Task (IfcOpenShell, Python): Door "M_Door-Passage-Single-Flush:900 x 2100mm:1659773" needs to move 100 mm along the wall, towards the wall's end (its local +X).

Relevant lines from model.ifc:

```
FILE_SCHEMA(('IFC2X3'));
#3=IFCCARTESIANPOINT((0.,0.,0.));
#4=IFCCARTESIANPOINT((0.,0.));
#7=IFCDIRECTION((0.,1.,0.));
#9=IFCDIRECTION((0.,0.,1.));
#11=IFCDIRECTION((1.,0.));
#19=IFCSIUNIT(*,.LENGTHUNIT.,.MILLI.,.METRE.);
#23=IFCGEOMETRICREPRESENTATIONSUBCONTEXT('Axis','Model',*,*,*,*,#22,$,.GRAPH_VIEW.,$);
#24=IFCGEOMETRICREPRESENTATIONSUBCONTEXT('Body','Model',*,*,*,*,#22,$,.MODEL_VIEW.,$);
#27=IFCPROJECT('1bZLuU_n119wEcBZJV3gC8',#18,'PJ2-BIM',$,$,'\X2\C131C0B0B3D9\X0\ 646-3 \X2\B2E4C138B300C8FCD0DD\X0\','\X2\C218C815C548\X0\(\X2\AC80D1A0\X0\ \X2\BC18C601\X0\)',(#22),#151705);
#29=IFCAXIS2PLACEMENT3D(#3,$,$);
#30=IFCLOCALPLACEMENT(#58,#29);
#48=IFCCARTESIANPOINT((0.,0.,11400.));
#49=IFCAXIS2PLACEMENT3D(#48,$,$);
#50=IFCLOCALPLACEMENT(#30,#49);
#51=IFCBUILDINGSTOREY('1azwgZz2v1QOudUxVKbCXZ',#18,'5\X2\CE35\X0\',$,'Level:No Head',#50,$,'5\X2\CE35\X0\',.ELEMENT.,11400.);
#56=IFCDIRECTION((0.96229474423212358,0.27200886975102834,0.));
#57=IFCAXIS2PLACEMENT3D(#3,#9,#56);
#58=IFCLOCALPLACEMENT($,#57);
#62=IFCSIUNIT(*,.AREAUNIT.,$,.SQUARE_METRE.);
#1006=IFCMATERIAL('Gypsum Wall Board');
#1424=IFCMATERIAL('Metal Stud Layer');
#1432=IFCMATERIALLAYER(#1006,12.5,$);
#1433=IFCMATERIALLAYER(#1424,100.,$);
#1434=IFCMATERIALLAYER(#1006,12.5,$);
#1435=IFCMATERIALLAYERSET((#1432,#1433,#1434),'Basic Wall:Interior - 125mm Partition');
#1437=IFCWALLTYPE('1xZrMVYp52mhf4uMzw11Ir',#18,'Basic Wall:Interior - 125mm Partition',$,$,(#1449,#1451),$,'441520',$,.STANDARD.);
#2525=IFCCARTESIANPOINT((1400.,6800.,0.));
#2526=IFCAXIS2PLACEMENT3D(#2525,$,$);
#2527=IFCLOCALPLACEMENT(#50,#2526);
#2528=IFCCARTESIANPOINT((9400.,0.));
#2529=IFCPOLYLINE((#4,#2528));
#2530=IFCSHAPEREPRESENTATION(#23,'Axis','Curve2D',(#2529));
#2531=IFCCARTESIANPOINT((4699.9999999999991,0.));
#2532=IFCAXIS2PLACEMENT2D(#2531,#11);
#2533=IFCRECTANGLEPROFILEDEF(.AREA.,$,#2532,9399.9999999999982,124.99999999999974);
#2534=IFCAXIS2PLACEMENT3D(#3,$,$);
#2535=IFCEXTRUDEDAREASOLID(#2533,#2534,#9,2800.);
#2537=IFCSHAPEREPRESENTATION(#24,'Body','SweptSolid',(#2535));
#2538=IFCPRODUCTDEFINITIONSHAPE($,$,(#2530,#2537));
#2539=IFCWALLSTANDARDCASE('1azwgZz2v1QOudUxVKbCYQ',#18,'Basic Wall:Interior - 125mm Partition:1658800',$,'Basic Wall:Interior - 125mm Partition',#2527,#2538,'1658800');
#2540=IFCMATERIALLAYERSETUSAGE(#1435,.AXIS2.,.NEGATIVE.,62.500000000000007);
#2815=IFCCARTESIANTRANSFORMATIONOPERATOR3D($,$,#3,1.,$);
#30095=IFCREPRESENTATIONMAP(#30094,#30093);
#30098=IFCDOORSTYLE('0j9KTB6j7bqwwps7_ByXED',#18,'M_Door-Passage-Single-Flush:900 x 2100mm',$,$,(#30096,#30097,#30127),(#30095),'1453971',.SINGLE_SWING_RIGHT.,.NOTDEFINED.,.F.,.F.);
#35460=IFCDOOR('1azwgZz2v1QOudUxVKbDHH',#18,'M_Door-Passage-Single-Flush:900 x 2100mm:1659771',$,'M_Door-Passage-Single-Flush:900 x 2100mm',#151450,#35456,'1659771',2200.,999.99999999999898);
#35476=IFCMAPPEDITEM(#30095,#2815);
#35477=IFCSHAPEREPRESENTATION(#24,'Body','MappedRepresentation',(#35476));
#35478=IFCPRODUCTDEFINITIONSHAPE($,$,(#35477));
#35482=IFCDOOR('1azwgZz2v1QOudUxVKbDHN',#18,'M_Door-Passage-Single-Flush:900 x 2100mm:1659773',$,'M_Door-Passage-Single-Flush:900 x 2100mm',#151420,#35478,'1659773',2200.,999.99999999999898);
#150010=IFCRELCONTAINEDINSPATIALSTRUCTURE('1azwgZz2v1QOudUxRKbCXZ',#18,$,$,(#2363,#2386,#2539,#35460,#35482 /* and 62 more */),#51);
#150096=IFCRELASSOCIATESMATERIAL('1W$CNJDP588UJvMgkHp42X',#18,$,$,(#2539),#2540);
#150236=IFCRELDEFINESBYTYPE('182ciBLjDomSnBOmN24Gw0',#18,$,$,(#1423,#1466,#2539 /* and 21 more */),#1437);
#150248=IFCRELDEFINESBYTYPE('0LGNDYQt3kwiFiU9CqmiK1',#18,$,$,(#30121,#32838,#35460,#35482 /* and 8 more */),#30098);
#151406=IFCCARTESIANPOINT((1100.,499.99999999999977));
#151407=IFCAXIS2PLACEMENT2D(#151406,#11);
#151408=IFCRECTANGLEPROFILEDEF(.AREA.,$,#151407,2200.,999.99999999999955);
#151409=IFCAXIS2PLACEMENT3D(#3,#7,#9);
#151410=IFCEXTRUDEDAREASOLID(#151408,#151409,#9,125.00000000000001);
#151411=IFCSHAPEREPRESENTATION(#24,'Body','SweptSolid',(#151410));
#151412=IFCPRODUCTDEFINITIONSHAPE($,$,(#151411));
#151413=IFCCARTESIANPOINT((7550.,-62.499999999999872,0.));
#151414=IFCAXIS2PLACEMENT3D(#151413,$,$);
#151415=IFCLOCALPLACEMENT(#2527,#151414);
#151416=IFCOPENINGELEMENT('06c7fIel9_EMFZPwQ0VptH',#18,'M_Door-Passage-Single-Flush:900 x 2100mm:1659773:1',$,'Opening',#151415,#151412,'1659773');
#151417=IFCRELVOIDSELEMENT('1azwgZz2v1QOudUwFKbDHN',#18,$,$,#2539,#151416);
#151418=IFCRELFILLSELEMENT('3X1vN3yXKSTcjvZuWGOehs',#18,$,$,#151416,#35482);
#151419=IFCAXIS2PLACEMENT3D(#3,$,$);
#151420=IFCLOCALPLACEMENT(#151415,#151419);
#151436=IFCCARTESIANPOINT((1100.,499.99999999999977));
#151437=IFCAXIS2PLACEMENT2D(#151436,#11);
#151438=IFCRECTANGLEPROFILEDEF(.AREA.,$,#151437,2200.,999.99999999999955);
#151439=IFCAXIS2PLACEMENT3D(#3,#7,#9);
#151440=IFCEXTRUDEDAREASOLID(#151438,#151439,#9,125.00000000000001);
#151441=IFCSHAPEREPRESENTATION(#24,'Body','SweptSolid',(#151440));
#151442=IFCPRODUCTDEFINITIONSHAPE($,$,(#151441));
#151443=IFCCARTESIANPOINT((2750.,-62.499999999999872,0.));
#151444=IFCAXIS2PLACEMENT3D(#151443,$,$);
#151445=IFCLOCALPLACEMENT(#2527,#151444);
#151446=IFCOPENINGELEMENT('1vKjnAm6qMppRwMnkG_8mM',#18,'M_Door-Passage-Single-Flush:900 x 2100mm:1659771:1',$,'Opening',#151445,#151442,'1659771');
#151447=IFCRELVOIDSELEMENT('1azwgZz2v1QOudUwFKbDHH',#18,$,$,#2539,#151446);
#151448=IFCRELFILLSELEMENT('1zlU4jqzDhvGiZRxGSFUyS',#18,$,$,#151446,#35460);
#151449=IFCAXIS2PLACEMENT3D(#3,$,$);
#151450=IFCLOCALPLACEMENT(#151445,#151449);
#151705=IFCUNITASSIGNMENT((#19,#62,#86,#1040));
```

```python
import ifcopenshell
import ifcopenshell.api.geometry
import ifcopenshell.util.placement

model = ifcopenshell.open("model.ifc")

door = model.by_guid("1azwgZz2v1QOudUxVKbDHN")
opening = door.FillsVoids[0].RelatingOpeningElement
wall = opening.VoidsElements[0].RelatingBuildingElement

wall_matrix = ifcopenshell.util.placement.get_local_placement(wall.ObjectPlacement)
shift = wall_matrix[:3, 0] * 100.0
before = ifcopenshell.util.placement.get_local_placement(door.ObjectPlacement)[:3, 3].copy()

# The door is placed relative to its opening, so it follows when the opening moves.
matrix = ifcopenshell.util.placement.get_local_placement(opening.ObjectPlacement)
matrix[:3, 3] += shift
ifcopenshell.api.geometry.edit_object_placement(
    model, product=opening, matrix=matrix, is_si=False, should_transform_children=True
)

after = ifcopenshell.util.placement.get_local_placement(door.ObjectPlacement)[:3, 3]
print("door moved by", (after - before).round(3) + 0.0)

model.write("model_edited.ifc")
```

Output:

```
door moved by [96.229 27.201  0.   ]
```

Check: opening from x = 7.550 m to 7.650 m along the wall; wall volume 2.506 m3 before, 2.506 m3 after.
